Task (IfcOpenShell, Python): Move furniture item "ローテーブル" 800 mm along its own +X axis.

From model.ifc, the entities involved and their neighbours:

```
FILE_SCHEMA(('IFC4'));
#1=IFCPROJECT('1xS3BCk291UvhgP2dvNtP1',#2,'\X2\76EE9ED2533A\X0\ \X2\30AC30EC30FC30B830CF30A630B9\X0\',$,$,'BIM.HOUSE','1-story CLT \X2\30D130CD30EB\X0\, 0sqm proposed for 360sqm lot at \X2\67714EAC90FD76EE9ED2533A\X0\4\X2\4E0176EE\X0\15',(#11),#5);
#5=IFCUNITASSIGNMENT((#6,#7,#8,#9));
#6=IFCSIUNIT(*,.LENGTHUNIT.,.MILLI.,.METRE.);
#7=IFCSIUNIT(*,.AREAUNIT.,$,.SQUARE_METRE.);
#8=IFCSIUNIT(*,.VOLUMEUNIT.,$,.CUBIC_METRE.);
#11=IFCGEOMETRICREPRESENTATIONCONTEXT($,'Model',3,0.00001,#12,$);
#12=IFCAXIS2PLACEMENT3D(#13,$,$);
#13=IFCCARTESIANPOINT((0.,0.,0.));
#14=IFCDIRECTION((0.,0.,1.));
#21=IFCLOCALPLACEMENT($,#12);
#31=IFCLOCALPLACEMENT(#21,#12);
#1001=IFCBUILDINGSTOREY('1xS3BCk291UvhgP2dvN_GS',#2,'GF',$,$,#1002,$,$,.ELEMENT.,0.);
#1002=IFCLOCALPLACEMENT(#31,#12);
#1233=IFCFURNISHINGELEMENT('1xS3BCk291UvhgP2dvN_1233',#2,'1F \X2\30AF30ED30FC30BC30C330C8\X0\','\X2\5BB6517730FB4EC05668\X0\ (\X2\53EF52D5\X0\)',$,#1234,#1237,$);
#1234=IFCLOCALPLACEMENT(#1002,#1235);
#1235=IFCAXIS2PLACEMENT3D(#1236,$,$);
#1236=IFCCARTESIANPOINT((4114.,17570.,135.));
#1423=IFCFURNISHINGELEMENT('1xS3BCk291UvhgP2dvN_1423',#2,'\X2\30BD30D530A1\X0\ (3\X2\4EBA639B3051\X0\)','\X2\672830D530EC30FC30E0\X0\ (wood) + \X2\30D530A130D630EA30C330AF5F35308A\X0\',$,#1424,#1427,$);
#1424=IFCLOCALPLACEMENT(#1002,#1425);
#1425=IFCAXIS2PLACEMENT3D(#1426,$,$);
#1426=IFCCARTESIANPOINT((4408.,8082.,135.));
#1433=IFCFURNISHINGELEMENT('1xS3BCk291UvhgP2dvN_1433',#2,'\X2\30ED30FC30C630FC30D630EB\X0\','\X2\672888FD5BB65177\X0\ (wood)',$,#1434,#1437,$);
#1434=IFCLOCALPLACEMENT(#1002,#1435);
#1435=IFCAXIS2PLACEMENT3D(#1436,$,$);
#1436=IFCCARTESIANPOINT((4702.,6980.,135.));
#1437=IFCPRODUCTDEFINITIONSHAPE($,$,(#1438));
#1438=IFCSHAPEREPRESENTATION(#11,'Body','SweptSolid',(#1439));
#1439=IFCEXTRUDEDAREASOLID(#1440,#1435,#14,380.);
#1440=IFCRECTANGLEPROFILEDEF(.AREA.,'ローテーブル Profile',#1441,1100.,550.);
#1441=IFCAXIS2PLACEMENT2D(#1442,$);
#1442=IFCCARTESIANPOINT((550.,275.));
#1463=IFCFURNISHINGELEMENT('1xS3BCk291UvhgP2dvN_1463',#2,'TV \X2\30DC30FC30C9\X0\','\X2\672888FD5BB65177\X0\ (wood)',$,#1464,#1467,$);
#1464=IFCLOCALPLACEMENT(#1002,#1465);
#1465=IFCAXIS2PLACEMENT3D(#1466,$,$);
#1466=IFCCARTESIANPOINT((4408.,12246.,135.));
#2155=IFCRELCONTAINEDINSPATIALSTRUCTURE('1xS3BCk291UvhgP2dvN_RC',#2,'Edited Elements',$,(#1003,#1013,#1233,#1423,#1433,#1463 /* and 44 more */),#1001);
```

```python
import ifcopenshell
import ifcopenshell.api.geometry
import ifcopenshell.util.placement
import ifcopenshell.util.unit

model = ifcopenshell.open("model.ifc")
unit_scale = ifcopenshell.util.unit.calculate_unit_scale(model)

item = model.by_guid("1xS3BCk291UvhgP2dvN_1433")
matrix = ifcopenshell.util.placement.get_local_placement(item.ObjectPlacement)
matrix[:3, 3] += matrix[:3, 0] * 0.8 / unit_scale
ifcopenshell.api.geometry.edit_object_placement(model, product=item, matrix=matrix, is_si=False)

print(ifcopenshell.util.placement.get_local_placement(item.ObjectPlacement).round(3) + 0.0)

model.write("model_edited.ifc")
```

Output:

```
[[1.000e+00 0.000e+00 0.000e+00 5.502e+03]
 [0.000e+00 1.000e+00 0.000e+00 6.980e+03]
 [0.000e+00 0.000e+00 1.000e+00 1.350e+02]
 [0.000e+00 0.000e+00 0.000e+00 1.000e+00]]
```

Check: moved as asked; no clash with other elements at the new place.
